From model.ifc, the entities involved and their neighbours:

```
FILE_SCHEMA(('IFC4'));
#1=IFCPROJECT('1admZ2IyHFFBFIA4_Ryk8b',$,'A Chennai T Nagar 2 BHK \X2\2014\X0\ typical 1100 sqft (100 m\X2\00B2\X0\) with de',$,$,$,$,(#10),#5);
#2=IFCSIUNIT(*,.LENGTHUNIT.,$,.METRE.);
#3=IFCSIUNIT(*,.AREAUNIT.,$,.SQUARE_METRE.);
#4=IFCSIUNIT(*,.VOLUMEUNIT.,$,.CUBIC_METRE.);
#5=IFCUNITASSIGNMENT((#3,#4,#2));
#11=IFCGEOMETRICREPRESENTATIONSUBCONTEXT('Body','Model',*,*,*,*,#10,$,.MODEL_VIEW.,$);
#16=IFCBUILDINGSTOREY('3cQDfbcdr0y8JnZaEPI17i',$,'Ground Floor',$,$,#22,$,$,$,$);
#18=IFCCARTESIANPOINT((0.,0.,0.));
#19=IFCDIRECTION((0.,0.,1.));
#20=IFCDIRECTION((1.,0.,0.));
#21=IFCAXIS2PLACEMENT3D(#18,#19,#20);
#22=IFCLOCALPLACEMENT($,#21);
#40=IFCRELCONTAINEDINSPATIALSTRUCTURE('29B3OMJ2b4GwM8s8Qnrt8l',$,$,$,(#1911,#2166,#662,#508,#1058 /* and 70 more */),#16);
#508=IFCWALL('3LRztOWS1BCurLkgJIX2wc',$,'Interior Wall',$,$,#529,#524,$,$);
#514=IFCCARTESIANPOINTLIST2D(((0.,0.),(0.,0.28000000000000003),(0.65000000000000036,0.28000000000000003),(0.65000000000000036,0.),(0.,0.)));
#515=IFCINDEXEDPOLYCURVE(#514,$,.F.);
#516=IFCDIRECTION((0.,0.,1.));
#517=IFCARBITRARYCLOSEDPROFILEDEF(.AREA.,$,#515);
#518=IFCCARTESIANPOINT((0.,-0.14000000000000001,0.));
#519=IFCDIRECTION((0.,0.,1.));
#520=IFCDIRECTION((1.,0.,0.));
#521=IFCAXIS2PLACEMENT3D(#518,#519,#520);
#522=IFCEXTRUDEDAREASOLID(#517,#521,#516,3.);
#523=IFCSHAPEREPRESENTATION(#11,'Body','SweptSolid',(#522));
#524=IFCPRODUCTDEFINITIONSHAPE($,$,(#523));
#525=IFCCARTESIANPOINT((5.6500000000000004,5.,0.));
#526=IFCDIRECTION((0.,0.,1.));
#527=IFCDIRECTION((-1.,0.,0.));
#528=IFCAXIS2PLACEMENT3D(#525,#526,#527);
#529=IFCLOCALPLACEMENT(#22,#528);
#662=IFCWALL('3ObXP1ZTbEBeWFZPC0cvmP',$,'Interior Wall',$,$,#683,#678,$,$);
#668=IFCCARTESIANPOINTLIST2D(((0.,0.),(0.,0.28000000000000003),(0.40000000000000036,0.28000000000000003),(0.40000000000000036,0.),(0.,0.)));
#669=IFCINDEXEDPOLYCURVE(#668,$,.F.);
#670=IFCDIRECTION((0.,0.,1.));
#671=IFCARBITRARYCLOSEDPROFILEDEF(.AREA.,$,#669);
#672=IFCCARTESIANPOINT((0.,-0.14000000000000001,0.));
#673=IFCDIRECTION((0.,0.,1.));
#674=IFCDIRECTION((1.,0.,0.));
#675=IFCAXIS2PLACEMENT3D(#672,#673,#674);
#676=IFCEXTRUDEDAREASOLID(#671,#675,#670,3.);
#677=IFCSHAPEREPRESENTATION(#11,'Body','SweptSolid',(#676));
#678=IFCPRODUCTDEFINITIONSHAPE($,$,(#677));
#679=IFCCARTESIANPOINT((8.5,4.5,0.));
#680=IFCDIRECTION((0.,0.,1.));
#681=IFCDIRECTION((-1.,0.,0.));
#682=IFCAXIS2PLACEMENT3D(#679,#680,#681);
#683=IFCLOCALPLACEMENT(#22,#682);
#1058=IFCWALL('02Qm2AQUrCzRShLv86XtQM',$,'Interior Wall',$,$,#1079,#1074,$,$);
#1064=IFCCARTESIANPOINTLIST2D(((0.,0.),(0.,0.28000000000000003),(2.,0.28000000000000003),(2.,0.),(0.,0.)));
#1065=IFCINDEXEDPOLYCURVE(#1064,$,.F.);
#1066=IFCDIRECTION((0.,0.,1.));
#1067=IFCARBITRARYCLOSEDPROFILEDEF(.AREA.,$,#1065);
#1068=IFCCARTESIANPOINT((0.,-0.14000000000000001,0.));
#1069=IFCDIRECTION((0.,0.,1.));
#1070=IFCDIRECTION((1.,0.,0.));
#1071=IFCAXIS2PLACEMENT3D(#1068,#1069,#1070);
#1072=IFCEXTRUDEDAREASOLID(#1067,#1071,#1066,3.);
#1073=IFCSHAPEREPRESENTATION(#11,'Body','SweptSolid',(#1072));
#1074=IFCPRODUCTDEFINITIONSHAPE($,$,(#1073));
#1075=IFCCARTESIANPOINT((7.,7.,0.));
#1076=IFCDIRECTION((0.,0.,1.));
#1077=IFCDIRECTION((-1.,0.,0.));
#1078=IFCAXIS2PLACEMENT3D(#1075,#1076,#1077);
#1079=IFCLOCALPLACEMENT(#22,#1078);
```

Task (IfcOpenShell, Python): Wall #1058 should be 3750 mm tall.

```python
import ifcopenshell
import ifcopenshell.geom
import ifcopenshell.util.representation
import ifcopenshell.util.shape
import ifcopenshell.util.unit

model = ifcopenshell.open("model.ifc")
unit_scale = ifcopenshell.util.unit.calculate_unit_scale(model)
settings = ifcopenshell.geom.settings()


def volume(element):
    """Net volume in cubic metres, openings subtracted."""
    shape = ifcopenshell.geom.create_shape(settings, element)
    return ifcopenshell.util.shape.get_volume(shape.geometry)


wall = model.by_guid("02Qm2AQUrCzRShLv86XtQM")
before = volume(wall)

body = ifcopenshell.util.representation.get_representation(wall, "Model", "Body")
solid = body.Items[0]
old_height = solid.Depth
solid.Depth = 3.75 / unit_scale
after = volume(wall)

print(f"height {old_height:g} -> {solid.Depth:g}, volume {before:.3f} -> {after:.3f} m3")

model.write("model-out.ifc")
```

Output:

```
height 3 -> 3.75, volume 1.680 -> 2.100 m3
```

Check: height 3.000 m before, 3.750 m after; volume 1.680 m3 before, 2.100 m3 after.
